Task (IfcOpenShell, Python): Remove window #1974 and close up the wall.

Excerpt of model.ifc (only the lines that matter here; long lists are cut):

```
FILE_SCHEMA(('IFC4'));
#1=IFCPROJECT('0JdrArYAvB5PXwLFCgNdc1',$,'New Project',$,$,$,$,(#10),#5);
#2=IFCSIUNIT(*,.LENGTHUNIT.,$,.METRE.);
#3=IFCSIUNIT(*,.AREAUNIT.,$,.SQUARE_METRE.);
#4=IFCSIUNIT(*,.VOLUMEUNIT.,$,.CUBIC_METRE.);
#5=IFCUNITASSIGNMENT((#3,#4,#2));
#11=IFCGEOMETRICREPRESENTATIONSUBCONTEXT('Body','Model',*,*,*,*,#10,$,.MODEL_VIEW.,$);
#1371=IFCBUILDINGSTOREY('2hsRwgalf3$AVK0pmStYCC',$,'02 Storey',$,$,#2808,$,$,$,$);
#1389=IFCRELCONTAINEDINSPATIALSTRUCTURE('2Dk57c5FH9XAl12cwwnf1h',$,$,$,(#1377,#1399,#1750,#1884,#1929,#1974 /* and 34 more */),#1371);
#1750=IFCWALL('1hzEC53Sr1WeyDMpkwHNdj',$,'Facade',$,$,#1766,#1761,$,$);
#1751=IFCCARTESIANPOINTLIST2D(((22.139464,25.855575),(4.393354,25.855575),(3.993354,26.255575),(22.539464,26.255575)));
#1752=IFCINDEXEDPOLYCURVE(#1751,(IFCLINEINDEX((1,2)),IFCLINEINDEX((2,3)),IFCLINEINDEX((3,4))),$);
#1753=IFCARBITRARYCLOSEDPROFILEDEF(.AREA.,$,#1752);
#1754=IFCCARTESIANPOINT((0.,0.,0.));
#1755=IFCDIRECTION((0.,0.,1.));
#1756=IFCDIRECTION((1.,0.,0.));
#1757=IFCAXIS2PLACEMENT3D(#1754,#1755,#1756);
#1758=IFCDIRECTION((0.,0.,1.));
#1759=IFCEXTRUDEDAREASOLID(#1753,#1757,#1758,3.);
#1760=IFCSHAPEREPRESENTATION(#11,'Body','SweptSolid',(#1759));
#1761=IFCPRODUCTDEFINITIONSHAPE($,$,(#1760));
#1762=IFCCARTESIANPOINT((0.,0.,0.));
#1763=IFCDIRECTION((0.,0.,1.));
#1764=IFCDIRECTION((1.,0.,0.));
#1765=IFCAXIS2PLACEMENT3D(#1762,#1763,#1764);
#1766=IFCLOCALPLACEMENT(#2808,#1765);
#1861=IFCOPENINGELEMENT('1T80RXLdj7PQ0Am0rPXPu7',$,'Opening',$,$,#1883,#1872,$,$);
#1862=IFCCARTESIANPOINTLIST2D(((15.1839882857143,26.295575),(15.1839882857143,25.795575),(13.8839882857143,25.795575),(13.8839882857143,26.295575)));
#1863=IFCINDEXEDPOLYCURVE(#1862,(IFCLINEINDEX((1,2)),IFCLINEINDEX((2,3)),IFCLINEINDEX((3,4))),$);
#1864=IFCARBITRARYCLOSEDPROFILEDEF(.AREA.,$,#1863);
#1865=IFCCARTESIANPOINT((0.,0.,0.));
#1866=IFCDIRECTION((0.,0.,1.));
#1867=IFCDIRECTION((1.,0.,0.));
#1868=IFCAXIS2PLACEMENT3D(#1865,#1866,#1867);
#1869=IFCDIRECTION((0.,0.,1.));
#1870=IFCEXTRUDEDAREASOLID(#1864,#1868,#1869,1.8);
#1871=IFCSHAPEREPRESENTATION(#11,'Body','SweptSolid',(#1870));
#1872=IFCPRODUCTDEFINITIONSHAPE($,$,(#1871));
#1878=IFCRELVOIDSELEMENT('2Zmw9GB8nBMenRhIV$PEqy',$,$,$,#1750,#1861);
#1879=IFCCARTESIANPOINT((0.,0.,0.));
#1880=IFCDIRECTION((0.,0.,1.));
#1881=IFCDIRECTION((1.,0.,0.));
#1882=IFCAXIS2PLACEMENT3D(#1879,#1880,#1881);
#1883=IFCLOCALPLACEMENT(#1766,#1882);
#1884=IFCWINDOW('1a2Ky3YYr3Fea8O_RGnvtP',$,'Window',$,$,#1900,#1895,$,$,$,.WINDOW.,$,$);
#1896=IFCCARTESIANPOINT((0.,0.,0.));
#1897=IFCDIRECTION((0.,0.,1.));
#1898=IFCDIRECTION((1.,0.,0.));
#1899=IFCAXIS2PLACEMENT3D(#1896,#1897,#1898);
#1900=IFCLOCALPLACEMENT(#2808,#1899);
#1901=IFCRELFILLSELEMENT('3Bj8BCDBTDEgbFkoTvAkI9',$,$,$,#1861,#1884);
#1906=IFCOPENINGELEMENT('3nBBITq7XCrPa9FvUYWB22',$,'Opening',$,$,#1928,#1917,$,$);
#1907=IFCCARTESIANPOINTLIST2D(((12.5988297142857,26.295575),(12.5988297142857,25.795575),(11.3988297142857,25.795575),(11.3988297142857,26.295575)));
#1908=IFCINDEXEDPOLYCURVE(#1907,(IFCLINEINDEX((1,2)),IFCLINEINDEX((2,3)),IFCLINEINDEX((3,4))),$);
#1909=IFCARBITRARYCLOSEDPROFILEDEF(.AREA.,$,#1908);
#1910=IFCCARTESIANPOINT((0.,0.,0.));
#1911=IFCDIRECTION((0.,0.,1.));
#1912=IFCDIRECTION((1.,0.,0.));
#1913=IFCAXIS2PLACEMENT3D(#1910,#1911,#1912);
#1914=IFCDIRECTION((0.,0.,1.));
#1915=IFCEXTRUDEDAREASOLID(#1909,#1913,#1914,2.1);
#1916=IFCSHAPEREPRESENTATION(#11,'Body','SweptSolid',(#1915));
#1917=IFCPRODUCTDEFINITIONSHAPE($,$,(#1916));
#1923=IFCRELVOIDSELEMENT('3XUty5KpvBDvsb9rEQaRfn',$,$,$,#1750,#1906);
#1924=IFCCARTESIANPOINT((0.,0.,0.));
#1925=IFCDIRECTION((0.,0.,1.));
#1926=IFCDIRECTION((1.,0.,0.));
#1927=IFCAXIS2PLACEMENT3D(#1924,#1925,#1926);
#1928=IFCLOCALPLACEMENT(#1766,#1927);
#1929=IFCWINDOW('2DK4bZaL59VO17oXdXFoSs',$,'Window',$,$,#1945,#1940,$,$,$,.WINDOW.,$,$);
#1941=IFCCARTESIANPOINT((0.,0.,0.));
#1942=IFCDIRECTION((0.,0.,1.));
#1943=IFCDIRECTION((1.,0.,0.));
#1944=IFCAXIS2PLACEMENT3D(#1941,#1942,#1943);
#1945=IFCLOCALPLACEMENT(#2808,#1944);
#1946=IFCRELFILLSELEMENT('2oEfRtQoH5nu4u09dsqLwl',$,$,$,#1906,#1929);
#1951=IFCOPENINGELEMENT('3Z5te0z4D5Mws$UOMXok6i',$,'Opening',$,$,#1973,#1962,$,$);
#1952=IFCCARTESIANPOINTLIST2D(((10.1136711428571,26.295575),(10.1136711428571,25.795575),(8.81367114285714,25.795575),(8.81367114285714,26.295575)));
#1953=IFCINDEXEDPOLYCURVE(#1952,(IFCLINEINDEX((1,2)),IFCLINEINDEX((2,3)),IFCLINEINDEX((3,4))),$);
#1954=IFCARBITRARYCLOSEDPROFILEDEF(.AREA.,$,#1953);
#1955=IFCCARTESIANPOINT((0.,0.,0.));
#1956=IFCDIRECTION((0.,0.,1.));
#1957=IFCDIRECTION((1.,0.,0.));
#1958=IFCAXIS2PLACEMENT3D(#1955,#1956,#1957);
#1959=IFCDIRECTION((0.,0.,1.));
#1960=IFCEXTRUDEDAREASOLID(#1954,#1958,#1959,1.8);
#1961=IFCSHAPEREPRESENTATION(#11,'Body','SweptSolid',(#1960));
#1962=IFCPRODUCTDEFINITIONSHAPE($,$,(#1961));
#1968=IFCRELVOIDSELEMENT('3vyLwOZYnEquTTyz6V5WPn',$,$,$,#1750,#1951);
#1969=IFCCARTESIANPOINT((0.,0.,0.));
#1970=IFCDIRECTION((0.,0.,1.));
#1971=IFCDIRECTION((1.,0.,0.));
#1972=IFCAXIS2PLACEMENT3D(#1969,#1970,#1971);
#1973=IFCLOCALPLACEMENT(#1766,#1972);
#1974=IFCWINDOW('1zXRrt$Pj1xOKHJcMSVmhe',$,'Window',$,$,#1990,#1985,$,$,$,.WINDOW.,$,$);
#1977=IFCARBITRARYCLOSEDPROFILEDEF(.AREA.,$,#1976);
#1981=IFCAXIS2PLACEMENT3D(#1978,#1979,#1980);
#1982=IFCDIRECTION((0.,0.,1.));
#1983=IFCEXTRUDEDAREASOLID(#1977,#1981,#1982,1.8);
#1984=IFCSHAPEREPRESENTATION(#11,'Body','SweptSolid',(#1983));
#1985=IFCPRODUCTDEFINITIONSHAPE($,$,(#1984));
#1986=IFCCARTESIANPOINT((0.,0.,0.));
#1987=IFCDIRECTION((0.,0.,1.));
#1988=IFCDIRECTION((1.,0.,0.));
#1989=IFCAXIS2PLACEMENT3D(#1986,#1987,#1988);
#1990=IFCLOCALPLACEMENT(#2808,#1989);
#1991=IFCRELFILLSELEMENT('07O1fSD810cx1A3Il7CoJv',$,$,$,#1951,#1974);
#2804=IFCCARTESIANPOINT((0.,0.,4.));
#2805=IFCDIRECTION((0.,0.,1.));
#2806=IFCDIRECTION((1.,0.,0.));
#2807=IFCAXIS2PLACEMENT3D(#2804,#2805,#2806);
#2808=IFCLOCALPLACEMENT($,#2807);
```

```python
import ifcopenshell
import ifcopenshell.api.feature
import ifcopenshell.api.root
import ifcopenshell.geom
import ifcopenshell.util.shape

model = ifcopenshell.open("model.ifc")
settings = ifcopenshell.geom.settings()


def volume(element):
    """Net volume in cubic metres, openings subtracted."""
    shape = ifcopenshell.geom.create_shape(settings, element)
    return ifcopenshell.util.shape.get_volume(shape.geometry)


window = model.by_guid("1zXRrt$Pj1xOKHJcMSVmhe")
opening = window.FillsVoids[0].RelatingOpeningElement
wall = opening.VoidsElements[0].RelatingBuildingElement
before = volume(wall)

ifcopenshell.api.root.remove_product(model, product=window)
ifcopenshell.api.feature.remove_feature(model, feature=opening)

after = volume(wall)

print(f"wall volume {before:.3f} -> {after:.3f} m3")

model.write("model_v2.ifc")
```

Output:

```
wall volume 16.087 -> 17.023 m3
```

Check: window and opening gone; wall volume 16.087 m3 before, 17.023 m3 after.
